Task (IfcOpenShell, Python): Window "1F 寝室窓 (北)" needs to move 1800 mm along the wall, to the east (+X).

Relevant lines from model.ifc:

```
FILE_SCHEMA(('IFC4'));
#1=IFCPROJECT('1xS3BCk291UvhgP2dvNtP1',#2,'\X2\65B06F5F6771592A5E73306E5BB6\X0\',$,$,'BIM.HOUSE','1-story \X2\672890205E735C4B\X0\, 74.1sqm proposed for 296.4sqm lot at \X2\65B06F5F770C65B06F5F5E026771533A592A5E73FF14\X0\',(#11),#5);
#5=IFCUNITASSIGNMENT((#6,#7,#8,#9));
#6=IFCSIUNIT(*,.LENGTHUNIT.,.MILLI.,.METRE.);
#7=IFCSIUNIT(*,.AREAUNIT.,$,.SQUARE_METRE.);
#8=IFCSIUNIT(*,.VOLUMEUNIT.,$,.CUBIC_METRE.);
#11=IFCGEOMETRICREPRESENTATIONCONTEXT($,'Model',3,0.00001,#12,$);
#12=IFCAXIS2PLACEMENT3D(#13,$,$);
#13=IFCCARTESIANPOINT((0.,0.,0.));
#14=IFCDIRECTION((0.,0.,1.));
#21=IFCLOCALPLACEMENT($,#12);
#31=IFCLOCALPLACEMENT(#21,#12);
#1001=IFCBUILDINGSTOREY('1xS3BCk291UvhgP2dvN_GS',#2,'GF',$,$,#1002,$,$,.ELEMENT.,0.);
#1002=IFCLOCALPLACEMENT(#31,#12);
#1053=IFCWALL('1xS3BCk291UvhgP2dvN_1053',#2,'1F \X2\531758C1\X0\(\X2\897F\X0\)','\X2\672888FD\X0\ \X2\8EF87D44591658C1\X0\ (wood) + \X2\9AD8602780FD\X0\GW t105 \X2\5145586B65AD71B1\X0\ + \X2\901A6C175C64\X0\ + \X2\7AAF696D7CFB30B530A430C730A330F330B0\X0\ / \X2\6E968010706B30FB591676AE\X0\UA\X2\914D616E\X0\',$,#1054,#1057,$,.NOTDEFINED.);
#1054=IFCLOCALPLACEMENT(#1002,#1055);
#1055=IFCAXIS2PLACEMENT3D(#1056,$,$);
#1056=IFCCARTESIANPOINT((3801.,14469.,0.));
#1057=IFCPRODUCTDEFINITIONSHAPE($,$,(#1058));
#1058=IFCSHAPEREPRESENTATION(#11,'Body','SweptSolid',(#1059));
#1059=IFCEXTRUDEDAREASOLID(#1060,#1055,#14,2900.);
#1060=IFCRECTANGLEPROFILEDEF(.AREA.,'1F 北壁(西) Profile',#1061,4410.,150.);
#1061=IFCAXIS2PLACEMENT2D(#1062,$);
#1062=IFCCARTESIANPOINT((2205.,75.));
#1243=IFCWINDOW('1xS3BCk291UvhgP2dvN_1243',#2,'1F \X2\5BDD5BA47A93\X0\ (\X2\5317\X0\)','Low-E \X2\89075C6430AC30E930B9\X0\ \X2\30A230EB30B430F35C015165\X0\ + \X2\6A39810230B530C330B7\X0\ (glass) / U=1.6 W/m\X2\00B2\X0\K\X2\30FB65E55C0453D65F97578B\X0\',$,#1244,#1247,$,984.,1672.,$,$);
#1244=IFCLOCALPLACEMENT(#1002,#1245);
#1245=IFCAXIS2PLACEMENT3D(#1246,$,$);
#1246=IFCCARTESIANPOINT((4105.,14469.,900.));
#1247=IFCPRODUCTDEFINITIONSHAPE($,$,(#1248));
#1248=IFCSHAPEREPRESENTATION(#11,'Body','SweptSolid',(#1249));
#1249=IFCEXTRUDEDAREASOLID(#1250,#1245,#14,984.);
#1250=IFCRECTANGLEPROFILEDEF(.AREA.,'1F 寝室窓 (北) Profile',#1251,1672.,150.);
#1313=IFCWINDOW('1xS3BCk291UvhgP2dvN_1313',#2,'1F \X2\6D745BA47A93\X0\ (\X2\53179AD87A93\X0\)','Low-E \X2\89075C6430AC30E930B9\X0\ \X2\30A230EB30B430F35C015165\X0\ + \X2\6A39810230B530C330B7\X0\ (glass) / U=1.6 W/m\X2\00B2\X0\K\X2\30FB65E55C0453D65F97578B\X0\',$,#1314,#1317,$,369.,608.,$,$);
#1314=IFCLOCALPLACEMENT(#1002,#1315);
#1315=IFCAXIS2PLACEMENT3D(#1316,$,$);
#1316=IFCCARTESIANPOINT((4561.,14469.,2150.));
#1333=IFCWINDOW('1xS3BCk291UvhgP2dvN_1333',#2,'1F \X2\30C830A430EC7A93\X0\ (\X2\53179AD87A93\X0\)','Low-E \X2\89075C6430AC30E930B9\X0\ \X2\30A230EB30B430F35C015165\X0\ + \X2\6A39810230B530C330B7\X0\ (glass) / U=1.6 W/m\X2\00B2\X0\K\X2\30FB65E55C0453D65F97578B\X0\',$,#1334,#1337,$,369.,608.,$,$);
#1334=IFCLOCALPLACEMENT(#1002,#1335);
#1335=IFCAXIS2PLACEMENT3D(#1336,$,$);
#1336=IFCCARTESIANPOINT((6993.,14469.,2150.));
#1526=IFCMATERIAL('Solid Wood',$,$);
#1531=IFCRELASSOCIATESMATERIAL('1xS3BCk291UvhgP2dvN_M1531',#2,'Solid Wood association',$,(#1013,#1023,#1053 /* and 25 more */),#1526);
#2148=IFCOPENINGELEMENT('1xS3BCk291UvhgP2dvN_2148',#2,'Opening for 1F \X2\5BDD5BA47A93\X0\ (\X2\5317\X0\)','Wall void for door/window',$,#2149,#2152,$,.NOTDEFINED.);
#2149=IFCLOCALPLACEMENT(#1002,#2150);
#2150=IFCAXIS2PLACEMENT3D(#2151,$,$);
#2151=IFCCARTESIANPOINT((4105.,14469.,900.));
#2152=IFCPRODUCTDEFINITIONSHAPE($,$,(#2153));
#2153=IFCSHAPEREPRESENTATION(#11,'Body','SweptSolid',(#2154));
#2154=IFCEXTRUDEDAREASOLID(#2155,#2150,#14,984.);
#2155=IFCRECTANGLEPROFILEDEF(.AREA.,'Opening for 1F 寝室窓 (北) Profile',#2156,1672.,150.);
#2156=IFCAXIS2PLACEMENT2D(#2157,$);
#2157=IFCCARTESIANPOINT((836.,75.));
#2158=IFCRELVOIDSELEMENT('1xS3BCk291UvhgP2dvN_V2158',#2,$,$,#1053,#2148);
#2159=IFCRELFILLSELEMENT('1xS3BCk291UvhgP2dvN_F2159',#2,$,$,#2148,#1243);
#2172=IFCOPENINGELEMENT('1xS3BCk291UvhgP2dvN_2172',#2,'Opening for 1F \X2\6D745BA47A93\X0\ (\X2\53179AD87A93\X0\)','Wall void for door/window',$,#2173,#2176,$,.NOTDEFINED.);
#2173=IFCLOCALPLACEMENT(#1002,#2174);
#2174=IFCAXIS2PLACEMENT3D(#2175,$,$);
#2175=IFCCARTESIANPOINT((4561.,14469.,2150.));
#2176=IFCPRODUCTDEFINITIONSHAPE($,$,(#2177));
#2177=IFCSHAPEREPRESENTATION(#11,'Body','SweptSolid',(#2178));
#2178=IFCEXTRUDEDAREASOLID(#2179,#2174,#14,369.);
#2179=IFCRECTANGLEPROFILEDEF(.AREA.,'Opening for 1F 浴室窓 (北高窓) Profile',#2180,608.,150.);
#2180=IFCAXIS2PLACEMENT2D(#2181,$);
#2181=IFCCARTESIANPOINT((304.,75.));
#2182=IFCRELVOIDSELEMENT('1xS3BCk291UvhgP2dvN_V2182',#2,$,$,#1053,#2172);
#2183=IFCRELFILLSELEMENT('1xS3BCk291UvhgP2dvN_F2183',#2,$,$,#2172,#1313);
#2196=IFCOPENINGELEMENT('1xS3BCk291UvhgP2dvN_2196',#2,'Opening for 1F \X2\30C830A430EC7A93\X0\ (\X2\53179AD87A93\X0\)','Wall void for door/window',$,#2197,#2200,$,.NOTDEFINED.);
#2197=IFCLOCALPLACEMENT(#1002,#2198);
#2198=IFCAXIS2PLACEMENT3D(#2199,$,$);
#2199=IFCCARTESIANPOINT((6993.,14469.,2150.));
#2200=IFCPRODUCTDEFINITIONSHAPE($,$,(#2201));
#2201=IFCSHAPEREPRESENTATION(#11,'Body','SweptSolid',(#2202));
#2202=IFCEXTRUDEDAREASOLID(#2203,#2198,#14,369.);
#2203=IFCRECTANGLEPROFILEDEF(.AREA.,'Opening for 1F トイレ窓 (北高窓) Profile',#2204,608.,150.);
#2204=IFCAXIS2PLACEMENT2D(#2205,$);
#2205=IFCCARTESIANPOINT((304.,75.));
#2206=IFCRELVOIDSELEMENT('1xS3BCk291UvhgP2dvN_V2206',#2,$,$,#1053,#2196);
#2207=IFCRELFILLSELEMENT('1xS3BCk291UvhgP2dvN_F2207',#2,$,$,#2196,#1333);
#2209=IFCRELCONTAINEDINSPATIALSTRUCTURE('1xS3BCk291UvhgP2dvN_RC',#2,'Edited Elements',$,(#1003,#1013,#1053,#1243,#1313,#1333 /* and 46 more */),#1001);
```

```python
import ifcopenshell
import ifcopenshell.api.geometry
import ifcopenshell.util.placement

model = ifcopenshell.open("model.ifc")

window = model.by_guid("1xS3BCk291UvhgP2dvN_1243")
opening = window.FillsVoids[0].RelatingOpeningElement
wall = opening.VoidsElements[0].RelatingBuildingElement

wall_matrix = ifcopenshell.util.placement.get_local_placement(wall.ObjectPlacement)
shift = wall_matrix[:3, 0] * 1800.0
before = ifcopenshell.util.placement.get_local_placement(window.ObjectPlacement)[:3, 3].copy()

# The window is not placed relative to its opening, so move both.
for product in (opening, window):
    matrix = ifcopenshell.util.placement.get_local_placement(product.ObjectPlacement)
    matrix[:3, 3] += shift
    ifcopenshell.api.geometry.edit_object_placement(model, product=product, matrix=matrix, is_si=False)

after = ifcopenshell.util.placement.get_local_placement(window.ObjectPlacement)[:3, 3]
print("window moved by", (after - before).round(3) + 0.0)

model.write("model-out.ifc")
```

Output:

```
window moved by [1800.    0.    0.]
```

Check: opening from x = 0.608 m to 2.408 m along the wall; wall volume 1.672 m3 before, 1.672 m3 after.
